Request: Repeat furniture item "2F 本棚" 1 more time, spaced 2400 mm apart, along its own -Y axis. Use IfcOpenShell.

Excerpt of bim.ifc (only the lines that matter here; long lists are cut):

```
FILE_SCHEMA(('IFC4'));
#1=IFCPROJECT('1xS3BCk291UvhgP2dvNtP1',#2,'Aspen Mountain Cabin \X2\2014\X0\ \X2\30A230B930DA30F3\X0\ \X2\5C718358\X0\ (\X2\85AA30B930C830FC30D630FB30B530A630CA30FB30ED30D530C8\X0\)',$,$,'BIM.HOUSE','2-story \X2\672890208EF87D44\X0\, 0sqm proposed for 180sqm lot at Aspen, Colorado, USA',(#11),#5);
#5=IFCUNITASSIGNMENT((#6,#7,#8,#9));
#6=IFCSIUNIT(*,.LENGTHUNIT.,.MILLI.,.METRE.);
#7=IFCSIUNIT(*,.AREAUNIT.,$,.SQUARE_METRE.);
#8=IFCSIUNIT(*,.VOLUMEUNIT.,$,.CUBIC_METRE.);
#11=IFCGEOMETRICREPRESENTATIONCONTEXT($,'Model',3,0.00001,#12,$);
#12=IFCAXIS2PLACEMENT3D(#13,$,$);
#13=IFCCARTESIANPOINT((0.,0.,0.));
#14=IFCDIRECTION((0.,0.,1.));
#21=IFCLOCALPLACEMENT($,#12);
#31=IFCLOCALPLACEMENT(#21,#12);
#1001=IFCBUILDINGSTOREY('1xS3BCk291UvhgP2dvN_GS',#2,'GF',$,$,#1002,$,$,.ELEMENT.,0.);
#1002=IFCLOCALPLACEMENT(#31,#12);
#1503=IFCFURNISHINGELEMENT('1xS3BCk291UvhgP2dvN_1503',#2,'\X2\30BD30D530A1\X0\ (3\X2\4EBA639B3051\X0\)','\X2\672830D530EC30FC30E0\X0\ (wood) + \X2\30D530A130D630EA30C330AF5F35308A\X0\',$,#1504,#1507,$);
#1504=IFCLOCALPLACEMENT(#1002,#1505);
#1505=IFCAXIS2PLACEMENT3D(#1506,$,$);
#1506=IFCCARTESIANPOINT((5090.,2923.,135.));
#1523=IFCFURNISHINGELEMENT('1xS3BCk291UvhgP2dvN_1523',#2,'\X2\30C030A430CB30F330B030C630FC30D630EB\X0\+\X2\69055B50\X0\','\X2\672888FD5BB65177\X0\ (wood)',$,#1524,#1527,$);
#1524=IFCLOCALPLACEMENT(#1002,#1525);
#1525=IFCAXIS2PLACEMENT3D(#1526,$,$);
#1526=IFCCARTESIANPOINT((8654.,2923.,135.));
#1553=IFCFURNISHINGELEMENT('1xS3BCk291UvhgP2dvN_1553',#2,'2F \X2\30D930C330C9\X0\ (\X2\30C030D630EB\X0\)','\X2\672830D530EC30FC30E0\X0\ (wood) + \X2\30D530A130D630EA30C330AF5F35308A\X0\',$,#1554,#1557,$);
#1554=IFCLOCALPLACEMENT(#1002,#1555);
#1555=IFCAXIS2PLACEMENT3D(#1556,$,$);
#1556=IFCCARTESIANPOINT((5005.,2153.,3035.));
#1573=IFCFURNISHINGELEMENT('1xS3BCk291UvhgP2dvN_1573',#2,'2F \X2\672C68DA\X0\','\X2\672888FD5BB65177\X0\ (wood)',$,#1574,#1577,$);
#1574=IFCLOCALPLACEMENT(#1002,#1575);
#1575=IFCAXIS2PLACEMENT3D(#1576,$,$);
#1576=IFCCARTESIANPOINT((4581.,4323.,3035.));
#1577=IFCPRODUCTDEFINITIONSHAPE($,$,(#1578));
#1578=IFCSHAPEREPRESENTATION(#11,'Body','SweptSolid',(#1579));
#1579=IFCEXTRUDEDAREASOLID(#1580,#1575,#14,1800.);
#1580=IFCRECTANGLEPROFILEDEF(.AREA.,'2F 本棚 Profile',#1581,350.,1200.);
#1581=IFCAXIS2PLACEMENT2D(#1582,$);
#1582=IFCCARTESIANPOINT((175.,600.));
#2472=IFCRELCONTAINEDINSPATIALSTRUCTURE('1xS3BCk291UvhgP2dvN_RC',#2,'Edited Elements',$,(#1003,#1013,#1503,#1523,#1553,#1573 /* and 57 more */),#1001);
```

```python
import ifcopenshell
import ifcopenshell.api.geometry
import ifcopenshell.api.root
import ifcopenshell.util.element
import ifcopenshell.util.placement
import ifcopenshell.util.unit

model = ifcopenshell.open("bim.ifc")
unit_scale = ifcopenshell.util.unit.calculate_unit_scale(model)


def reuse_history(source, copy):
    """copy_class also copies each property set's owner history, people and application; keep the originals."""
    for rel in copy.IsDefinedBy:
        if rel.is_a("IfcRelDefinesByProperties") and (history := rel.RelatingPropertyDefinition.OwnerHistory):
            rel.RelatingPropertyDefinition.OwnerHistory = source.OwnerHistory
            ifcopenshell.util.element.remove_deep2(model, history)


source = model.by_id(1573)
base = ifcopenshell.util.placement.get_local_placement(source.ObjectPlacement)
step = -base[:3, 1] * 2.4 / unit_scale

for i in range(1, 2):
    copy = ifcopenshell.api.root.copy_class(model, product=source)
    copy.Representation = ifcopenshell.util.element.copy_deep(
        model, source.Representation, exclude=["IfcGeometricRepresentationContext", "IfcRepresentationMap"]
    )
    reuse_history(source, copy)
    matrix = base.copy()
    matrix[:3, 3] += i * step
    print("added at", matrix[:3, 3].round(3) + 0.0)
    ifcopenshell.api.geometry.edit_object_placement(model, product=copy, matrix=matrix, is_si=False)

model.write("bim_edited.ifc")
```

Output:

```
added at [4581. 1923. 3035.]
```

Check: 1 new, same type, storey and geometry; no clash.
